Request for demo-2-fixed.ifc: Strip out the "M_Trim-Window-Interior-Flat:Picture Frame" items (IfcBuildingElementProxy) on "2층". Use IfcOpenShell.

First a look at what the model holds.

```python
import ifcopenshell
import ifcopenshell.util.element

model = ifcopenshell.open("demo-2-fixed.ifc")
print(model.schema)
storey = next(s for s in model.by_type("IfcBuildingStorey") if s.Name == "2층")
proxies = [e for e in ifcopenshell.util.element.get_decomposition(storey) if e.is_a("IfcBuildingElementProxy")]
seen = {}
for e in proxies:
    element_type = ifcopenshell.util.element.get_type(e)
    name = element_type.Name if element_type not in (None, e) else None
    seen[name] = seen.get(name, 0) + 1
for name, count in sorted(seen.items(), key=str):
    print(count, "x", name)
```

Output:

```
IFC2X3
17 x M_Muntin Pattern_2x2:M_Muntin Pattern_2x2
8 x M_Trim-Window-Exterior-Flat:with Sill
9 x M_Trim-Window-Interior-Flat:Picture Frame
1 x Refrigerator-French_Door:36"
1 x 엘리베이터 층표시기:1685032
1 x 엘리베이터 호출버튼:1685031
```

```python
import ifcopenshell
import ifcopenshell.api.root
import ifcopenshell.util.element

model = ifcopenshell.open("demo-2-fixed.ifc")

storey = next(s for s in model.by_type("IfcBuildingStorey") if s.Name == "2층")
proxies = [e for e in ifcopenshell.util.element.get_decomposition(storey) if e.is_a("IfcBuildingElementProxy")]
targets = [e for e in proxies if (t := ifcopenshell.util.element.get_type(e)) not in (None, e) and t.Name == "M_Trim-Window-Interior-Flat:Picture Frame"]

for e in targets:
    ifcopenshell.api.root.remove_product(model, product=e)
print(len(targets), "removed")

model.write("demo-2-fixed-out.ifc")
```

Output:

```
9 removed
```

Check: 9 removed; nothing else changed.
